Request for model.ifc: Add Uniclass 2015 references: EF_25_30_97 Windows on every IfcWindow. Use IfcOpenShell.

First a look at what the model holds.

```python
import ifcopenshell

model = ifcopenshell.open("model.ifc")
print(model.schema)
print("classifications:", [c.Name for c in model.by_type("IfcClassification")])
for ifc_class in ("IfcDoor", "IfcRoof", "IfcStair", "IfcWall", "IfcWindow"):
    print(ifc_class, len(model.by_type(ifc_class)))
```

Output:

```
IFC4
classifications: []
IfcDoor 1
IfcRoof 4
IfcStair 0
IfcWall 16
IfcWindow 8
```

```python
import ifcopenshell
import ifcopenshell.api.classification

model = ifcopenshell.open("model.ifc")

system = ifcopenshell.api.classification.add_classification(model, classification="Uniclass 2015")

codes = {
    "IfcWindow": ("EF_25_30_97", "Windows"),
}
for ifc_class, (code, name) in codes.items():
    products = model.by_type(ifc_class)
    ifcopenshell.api.classification.add_reference(
        model, products=products, classification=system, identification=code, name=name
    )
    print(code, len(products))

model.write("model_edited.ifc")
```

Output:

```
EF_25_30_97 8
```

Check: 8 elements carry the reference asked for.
